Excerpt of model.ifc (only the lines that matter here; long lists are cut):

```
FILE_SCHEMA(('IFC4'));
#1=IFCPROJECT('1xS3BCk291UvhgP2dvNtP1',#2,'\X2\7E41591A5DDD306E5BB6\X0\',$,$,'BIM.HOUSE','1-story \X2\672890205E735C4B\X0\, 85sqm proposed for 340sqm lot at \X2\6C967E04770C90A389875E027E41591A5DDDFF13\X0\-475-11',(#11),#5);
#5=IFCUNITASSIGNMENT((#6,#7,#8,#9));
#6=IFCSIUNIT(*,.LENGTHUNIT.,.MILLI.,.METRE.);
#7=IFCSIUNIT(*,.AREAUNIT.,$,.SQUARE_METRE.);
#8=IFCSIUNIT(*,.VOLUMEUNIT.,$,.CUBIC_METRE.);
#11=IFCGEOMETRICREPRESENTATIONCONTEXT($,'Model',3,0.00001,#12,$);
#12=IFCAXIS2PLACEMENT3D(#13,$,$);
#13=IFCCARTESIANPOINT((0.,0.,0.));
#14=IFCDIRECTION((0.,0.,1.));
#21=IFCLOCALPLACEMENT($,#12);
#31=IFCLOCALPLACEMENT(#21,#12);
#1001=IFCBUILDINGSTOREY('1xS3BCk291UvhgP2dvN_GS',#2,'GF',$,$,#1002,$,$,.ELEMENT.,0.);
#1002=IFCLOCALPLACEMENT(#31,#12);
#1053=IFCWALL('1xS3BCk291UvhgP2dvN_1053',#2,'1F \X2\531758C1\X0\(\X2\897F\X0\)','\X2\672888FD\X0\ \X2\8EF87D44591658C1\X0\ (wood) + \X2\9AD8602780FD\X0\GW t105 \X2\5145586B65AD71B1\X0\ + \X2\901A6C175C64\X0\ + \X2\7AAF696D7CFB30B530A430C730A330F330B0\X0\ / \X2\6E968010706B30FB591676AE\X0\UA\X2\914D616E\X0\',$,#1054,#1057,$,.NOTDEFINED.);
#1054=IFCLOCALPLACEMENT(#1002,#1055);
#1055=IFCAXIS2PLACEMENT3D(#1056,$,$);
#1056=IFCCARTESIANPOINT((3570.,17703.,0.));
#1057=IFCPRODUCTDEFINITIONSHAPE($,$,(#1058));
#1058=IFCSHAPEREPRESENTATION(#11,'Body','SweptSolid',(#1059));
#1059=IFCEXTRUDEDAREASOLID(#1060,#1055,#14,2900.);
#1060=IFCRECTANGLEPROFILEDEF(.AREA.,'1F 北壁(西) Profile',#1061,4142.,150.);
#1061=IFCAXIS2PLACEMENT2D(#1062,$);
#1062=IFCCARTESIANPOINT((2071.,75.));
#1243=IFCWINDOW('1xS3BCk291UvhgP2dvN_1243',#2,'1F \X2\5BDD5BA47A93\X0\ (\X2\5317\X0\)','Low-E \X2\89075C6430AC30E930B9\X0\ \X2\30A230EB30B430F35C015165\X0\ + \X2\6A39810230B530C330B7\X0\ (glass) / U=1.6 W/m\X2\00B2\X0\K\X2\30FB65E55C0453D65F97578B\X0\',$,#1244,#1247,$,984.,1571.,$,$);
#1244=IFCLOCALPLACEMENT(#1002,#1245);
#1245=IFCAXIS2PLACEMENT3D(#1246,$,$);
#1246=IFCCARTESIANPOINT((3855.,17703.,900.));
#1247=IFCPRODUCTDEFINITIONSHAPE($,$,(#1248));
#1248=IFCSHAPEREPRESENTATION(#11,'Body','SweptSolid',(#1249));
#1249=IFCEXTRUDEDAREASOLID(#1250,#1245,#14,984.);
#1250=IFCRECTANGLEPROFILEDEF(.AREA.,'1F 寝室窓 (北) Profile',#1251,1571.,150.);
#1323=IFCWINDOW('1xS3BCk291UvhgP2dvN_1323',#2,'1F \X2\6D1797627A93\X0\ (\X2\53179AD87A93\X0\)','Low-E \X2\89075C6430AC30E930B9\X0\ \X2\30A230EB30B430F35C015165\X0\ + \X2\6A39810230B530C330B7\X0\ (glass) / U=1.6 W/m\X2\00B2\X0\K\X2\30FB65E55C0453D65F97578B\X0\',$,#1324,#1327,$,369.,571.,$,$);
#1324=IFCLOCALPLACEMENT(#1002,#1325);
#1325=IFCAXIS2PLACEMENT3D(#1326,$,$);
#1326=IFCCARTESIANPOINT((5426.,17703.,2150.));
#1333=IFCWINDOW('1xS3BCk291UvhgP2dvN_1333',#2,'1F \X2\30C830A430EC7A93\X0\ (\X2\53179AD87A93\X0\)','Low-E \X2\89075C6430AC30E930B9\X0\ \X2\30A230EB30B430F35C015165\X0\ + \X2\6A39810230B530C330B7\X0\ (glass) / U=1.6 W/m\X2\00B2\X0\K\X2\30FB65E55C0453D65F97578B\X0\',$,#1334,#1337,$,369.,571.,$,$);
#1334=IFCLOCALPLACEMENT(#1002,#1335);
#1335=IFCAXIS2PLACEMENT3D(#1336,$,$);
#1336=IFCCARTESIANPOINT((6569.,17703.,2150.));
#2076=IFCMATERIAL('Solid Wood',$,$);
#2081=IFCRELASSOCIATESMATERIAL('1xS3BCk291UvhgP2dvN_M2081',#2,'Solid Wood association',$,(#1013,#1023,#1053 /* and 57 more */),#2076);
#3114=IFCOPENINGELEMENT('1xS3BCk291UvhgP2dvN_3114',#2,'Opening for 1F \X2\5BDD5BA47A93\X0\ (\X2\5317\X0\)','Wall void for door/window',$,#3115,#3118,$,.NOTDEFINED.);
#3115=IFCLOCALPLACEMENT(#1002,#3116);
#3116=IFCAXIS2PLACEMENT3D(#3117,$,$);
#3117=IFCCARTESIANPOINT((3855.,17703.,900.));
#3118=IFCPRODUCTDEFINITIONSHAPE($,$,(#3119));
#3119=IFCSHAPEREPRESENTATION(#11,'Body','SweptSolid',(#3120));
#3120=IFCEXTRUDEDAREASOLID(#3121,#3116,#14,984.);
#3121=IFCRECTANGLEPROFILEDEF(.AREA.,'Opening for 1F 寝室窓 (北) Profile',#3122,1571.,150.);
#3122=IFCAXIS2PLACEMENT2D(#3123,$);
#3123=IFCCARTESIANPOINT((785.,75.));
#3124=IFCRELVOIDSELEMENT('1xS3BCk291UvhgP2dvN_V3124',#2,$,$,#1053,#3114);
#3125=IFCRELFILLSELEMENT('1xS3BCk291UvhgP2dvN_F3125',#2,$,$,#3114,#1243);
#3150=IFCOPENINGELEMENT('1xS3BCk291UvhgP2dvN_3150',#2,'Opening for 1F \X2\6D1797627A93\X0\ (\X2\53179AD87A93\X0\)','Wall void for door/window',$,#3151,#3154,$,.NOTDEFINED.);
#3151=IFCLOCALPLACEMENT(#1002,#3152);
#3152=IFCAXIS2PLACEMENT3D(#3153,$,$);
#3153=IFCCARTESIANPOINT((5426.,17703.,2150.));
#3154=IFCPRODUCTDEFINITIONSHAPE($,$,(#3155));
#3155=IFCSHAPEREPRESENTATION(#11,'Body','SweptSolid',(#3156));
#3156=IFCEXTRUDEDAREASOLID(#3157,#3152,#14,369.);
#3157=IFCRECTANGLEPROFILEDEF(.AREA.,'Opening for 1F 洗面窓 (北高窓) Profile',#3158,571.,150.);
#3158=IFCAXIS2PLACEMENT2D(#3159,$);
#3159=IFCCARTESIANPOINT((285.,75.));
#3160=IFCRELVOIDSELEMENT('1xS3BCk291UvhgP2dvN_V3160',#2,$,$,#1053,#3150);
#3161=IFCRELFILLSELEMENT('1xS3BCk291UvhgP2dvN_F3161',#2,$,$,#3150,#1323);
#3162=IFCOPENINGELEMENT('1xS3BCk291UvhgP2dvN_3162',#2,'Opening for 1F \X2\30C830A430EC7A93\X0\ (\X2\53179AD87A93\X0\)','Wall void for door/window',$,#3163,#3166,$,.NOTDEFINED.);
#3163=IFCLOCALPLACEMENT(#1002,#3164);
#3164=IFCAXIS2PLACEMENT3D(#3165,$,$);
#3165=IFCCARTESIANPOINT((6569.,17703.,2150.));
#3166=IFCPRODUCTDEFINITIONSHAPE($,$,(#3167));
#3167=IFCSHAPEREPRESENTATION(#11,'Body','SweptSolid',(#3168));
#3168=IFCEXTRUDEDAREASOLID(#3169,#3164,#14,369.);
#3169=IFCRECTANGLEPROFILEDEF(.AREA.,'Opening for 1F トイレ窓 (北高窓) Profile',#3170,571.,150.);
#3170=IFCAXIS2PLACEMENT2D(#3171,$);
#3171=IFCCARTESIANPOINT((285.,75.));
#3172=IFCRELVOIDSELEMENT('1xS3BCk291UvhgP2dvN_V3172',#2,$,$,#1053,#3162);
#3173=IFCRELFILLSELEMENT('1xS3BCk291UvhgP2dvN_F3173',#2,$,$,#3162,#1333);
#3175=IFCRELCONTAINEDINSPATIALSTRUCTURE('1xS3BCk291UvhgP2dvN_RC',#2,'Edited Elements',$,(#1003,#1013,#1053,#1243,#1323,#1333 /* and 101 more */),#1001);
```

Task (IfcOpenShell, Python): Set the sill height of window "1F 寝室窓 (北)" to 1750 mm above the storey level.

```python
import numpy as np
import ifcopenshell
import ifcopenshell.api.geometry
import ifcopenshell.geom
import ifcopenshell.util.element
import ifcopenshell.util.placement
import ifcopenshell.util.shape
import ifcopenshell.util.unit

model = ifcopenshell.open("model.ifc")
unit_scale = ifcopenshell.util.unit.calculate_unit_scale(model)

window = model.by_id(1243)
opening = window.FillsVoids[0].RelatingOpeningElement
storey = ifcopenshell.util.element.get_container(window, ifc_class="IfcBuildingStorey")
level = ifcopenshell.util.placement.get_local_placement(storey.ObjectPlacement)[2, 3]

# The opening's origin need not be at the sill, so measure its lowest point.
shape = ifcopenshell.geom.create_shape(ifcopenshell.geom.settings(), opening)
bottom = ifcopenshell.util.shape.get_shape_bottom_elevation(shape, shape.geometry) / unit_scale
dz = level + 1.75 / unit_scale - bottom

shift = np.array([0.0, 0.0, dz])
# The window is not placed relative to its opening, so move both.
for product in (opening, window):
    matrix = ifcopenshell.util.placement.get_local_placement(product.ObjectPlacement)
    matrix[:3, 3] += shift
    ifcopenshell.api.geometry.edit_object_placement(model, product=product, matrix=matrix, is_si=False)

print(f"moved by {dz * unit_scale:+.3f} m")

model.write("model_v2.ifc")
```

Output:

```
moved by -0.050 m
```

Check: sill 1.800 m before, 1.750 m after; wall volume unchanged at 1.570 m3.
